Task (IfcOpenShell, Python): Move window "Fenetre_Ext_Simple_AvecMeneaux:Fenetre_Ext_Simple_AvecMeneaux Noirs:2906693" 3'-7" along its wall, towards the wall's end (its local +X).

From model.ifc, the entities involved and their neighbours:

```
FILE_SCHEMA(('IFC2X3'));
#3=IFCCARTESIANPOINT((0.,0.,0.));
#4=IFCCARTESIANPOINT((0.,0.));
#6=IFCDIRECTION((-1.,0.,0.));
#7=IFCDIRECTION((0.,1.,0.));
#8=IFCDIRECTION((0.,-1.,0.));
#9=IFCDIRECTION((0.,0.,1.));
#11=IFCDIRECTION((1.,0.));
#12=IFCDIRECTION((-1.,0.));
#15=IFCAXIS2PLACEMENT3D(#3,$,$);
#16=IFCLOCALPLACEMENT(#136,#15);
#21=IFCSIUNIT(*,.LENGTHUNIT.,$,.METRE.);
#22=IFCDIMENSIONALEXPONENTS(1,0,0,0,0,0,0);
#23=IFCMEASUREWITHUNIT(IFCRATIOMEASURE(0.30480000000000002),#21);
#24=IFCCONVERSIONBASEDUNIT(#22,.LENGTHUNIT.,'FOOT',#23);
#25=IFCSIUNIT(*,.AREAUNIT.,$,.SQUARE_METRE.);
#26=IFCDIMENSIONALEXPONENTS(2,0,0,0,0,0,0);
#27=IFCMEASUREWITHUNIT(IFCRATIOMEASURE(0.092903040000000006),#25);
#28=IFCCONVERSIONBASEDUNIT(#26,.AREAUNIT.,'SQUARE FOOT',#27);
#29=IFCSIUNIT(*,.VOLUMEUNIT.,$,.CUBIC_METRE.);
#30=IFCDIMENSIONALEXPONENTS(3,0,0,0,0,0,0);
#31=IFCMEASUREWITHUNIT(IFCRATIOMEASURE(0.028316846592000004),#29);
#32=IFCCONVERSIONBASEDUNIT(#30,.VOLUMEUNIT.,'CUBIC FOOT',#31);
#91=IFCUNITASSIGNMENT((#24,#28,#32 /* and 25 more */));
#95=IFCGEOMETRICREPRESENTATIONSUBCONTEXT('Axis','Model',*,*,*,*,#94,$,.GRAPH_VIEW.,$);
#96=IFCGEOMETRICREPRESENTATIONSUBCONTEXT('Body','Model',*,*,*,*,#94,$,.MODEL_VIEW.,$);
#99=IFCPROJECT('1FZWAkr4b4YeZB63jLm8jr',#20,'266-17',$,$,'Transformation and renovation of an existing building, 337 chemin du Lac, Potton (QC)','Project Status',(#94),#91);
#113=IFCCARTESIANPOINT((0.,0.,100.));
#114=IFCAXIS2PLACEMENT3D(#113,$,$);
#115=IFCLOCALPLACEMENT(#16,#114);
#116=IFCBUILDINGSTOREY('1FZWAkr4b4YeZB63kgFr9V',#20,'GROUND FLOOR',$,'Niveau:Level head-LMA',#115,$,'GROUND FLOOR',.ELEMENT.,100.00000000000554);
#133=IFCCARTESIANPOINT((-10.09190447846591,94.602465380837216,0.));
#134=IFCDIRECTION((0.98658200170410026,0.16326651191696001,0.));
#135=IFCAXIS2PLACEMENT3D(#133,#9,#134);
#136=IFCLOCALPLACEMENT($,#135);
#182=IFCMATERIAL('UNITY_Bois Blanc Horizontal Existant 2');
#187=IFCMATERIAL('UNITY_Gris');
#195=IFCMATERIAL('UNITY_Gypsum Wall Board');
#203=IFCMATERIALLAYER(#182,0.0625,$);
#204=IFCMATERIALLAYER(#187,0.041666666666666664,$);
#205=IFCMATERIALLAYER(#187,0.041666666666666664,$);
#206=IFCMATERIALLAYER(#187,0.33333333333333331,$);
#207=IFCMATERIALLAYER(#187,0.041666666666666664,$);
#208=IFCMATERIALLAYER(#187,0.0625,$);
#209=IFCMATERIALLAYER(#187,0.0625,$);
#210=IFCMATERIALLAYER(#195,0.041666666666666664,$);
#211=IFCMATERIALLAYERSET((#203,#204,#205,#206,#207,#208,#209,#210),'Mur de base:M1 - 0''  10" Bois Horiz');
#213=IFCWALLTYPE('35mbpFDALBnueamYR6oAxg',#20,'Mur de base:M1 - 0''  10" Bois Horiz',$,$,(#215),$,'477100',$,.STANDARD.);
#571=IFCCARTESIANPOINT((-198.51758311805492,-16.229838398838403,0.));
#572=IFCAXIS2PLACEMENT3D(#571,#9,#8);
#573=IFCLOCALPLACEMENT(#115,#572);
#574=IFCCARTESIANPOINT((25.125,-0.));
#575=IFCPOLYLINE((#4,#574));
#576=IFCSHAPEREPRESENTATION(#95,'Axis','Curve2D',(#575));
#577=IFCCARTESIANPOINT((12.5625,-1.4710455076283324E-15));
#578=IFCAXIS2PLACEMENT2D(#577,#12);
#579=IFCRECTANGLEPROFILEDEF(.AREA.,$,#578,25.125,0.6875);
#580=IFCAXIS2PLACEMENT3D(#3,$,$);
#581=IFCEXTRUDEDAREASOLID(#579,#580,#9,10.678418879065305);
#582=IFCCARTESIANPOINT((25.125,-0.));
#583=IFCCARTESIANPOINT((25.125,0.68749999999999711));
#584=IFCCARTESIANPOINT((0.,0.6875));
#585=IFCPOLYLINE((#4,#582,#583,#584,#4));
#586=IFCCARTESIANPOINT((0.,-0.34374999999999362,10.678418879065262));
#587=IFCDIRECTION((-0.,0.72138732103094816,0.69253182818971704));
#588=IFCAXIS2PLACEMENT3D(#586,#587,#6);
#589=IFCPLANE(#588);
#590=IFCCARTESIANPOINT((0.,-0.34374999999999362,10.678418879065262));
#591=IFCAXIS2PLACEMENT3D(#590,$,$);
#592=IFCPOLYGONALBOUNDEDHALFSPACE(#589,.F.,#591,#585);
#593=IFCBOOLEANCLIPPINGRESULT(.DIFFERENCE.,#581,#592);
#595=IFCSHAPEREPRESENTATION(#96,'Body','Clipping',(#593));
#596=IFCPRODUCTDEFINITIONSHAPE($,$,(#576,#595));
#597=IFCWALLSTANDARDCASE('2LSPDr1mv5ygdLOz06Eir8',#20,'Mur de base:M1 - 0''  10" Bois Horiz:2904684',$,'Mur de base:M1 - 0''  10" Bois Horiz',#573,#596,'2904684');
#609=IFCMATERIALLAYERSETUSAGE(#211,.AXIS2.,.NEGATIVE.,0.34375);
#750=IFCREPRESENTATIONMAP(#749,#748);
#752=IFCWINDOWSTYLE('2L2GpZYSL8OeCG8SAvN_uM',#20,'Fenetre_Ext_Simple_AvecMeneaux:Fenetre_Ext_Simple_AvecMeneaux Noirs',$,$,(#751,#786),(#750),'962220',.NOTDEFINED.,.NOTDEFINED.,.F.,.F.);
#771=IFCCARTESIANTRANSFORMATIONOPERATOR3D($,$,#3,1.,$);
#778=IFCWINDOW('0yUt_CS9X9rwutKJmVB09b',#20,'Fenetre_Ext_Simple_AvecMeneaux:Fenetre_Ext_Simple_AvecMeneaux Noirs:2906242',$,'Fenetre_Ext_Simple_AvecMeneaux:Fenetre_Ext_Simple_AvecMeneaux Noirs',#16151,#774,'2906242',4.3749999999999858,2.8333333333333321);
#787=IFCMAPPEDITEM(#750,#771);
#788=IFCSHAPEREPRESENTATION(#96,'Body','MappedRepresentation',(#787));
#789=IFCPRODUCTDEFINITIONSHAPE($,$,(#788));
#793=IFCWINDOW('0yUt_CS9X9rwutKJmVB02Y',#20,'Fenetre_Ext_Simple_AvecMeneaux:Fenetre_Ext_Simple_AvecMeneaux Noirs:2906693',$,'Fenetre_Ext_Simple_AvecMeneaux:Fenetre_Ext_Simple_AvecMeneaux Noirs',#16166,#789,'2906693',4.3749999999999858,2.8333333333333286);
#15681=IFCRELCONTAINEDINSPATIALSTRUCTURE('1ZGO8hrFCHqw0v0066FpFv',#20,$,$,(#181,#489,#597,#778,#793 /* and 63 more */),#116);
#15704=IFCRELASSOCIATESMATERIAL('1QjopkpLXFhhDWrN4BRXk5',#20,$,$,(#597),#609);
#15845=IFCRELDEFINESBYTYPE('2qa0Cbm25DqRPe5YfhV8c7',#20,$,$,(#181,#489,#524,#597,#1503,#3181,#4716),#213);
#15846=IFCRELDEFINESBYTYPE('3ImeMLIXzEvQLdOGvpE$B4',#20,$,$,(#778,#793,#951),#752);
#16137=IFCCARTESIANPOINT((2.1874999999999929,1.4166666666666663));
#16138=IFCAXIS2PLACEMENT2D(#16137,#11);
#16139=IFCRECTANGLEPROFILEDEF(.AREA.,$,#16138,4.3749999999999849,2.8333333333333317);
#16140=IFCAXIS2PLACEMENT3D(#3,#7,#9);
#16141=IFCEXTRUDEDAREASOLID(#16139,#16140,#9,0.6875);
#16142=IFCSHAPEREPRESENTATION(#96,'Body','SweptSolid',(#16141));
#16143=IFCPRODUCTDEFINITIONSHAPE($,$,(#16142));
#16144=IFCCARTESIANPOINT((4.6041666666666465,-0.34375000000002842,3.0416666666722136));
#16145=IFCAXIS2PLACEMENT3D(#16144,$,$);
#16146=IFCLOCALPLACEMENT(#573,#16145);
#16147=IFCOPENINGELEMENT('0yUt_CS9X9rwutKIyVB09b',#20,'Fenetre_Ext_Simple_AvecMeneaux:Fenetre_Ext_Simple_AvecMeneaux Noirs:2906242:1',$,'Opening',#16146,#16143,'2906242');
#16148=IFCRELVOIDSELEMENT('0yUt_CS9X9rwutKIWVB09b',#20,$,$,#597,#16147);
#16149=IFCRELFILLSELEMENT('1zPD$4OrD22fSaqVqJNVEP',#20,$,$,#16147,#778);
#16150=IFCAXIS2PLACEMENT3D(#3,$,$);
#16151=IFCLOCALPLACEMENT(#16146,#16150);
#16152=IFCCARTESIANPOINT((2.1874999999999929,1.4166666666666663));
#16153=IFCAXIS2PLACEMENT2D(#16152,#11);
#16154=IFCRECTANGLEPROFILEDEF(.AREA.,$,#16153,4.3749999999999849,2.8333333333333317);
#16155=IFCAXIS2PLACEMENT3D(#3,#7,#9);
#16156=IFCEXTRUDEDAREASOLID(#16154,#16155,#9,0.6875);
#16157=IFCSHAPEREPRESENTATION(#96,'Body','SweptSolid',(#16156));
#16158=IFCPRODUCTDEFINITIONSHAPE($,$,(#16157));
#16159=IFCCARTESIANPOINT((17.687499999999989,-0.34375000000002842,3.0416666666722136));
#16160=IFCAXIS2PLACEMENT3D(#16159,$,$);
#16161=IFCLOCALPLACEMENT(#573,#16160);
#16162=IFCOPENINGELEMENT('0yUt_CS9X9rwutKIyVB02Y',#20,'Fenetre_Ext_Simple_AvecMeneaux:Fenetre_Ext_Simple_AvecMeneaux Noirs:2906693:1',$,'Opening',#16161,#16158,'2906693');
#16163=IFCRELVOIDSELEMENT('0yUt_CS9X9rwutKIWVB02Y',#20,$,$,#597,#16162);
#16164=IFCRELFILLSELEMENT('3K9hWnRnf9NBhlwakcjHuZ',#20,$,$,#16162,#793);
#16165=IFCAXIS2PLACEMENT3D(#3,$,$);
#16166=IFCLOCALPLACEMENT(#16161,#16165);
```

```python
import ifcopenshell
import ifcopenshell.api.geometry
import ifcopenshell.util.placement
import ifcopenshell.util.unit

model = ifcopenshell.open("model.ifc")
unit_scale = ifcopenshell.util.unit.calculate_unit_scale(model)

window = model.by_guid("0yUt_CS9X9rwutKJmVB02Y")
opening = window.FillsVoids[0].RelatingOpeningElement
wall = opening.VoidsElements[0].RelatingBuildingElement

wall_matrix = ifcopenshell.util.placement.get_local_placement(wall.ObjectPlacement)
shift = wall_matrix[:3, 0] * 43 * 0.0254 / unit_scale
before = ifcopenshell.util.placement.get_local_placement(window.ObjectPlacement)[:3, 3].copy()

# The window is placed relative to its opening, so it follows when the opening moves.
matrix = ifcopenshell.util.placement.get_local_placement(opening.ObjectPlacement)
matrix[:3, 3] += shift
ifcopenshell.api.geometry.edit_object_placement(
    model, product=opening, matrix=matrix, is_si=False, should_transform_children=True
)

after = ifcopenshell.util.placement.get_local_placement(window.ObjectPlacement)[:3, 3]
print("window moved by", (after - before).round(3) + 0.0)

model.write("model_edited.ifc")
```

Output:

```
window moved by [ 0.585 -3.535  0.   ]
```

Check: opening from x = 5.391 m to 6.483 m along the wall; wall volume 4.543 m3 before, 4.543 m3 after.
